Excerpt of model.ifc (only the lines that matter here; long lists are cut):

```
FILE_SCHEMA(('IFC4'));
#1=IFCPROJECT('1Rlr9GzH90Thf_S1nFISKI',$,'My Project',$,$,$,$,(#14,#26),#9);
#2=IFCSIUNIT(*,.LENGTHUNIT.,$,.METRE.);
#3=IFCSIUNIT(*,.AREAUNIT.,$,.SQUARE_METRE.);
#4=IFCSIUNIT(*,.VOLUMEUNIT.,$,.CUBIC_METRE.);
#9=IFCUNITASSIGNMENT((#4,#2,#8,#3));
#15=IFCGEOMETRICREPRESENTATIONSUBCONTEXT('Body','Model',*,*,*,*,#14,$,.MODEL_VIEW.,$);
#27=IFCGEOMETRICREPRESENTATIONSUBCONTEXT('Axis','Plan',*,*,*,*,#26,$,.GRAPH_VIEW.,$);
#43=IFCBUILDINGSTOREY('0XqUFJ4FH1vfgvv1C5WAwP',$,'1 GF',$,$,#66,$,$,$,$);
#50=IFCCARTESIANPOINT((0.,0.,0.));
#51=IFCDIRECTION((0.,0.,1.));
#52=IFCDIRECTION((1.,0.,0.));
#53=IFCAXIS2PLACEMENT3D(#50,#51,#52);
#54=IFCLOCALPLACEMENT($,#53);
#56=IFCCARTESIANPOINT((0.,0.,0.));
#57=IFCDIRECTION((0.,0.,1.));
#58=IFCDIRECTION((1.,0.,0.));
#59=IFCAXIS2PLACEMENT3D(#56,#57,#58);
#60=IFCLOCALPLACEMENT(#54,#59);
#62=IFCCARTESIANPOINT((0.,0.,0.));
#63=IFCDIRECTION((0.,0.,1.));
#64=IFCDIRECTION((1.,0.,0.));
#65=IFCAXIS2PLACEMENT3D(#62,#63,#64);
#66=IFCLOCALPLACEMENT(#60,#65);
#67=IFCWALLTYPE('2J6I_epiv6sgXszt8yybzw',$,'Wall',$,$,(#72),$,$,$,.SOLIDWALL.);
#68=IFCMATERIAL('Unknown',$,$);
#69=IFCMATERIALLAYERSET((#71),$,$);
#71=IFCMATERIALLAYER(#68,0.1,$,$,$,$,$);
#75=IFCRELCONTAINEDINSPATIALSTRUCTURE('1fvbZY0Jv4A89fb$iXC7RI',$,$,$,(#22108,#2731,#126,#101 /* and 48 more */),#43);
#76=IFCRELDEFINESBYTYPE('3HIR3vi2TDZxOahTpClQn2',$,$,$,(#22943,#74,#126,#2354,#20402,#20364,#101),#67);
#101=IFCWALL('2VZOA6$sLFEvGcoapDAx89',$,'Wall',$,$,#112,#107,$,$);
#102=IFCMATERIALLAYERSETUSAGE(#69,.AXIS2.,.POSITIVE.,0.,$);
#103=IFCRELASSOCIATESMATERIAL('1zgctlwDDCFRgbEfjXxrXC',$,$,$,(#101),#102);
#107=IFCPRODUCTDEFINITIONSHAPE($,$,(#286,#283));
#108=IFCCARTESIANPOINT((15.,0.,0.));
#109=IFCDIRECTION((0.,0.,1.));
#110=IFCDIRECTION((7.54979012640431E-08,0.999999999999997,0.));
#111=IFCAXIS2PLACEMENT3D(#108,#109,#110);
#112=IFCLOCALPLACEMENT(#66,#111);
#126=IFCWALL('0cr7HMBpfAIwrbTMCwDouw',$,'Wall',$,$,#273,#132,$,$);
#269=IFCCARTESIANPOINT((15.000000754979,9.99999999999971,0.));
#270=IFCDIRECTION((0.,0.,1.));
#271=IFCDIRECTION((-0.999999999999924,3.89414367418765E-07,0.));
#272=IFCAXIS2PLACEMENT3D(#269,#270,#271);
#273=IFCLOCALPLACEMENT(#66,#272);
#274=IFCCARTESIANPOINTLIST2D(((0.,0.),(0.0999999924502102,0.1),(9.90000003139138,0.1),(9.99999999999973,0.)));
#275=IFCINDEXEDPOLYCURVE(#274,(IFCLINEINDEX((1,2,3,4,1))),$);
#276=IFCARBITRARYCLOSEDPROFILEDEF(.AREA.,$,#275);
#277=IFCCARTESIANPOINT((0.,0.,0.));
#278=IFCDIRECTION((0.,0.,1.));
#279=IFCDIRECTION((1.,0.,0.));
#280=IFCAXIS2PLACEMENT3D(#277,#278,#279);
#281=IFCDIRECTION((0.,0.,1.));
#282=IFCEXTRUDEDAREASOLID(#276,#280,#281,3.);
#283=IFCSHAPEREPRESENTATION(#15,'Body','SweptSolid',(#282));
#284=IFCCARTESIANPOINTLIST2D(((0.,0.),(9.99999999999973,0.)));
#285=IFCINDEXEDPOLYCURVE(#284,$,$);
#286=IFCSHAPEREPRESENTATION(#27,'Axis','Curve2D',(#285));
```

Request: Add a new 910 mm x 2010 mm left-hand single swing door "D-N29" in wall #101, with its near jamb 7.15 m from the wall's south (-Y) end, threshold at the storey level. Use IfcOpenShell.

```python
import numpy as np
import ifcopenshell
import ifcopenshell.api.feature
import ifcopenshell.api.geometry
import ifcopenshell.api.root
import ifcopenshell.api.spatial
import ifcopenshell.geom
import ifcopenshell.util.element
import ifcopenshell.util.placement
import ifcopenshell.util.representation
import ifcopenshell.util.shape
import ifcopenshell.util.unit

model = ifcopenshell.open("model.ifc")
unit_scale = ifcopenshell.util.unit.calculate_unit_scale(model)
settings = ifcopenshell.geom.settings()


def volume(element):
    """Net volume in cubic metres, openings subtracted."""
    shape = ifcopenshell.geom.create_shape(settings, element)
    return ifcopenshell.util.shape.get_volume(shape.geometry)


wall = model.by_guid("2VZOA6$sLFEvGcoapDAx89")
storey = ifcopenshell.util.element.get_container(wall, ifc_class="IfcBuildingStorey")
context = ifcopenshell.util.representation.get_context(model, "Model", "Body", "MODEL_VIEW")
before = volume(wall)

width, height, from_end, sill = 0.91, 2.01, 7.15, 0.0  # metres

# The wall runs along its own X axis, and the end named is its -X end.
wall_shape = ifcopenshell.geom.create_shape(settings, wall)
x, y, z = ifcopenshell.util.shape.get_vertices(wall_shape.geometry).T
start = x.min() + from_end
face, thickness = float(y.min()), float(y.max() - y.min())
wall_matrix = ifcopenshell.util.placement.get_local_placement(wall.ObjectPlacement)
level = ifcopenshell.util.placement.get_local_placement(storey.ObjectPlacement)[2, 3]


def in_wall(x, y):
    """Placement at x, y metres in the wall's axes, at sill height."""
    matrix = wall_matrix.copy()
    matrix[:, 3] = wall_matrix @ np.array([x / unit_scale, y / unit_scale, 0.0, 1.0])
    matrix[2, 3] = level + sill / unit_scale
    return matrix


# Opening: a box that overshoots both wall faces by 50 mm.
opening = ifcopenshell.api.root.create_entity(model, ifc_class="IfcOpeningElement", predefined_type="OPENING")
box = ifcopenshell.api.geometry.add_wall_representation(
    model, context=context, length=width, height=height, thickness=thickness + 0.1
)
ifcopenshell.api.geometry.assign_representation(model, product=opening, representation=box)
ifcopenshell.api.geometry.edit_object_placement(model, product=opening, matrix=in_wall(start, face - 0.05), is_si=False)
ifcopenshell.api.feature.add_feature(model, feature=opening, element=wall)

door = ifcopenshell.api.root.create_entity(model, ifc_class="IfcDoor", name="D-N29", predefined_type="DOOR")
door.OverallWidth, door.OverallHeight = width / unit_scale, height / unit_scale
door.OperationType = "SINGLE_SWING_LEFT"
body = ifcopenshell.api.geometry.add_door_representation(
    model,
    context=context,
    overall_width=door.OverallWidth,
    overall_height=door.OverallHeight,
    operation_type="SINGLE_SWING_LEFT",
    lining_properties={"LiningDepth": thickness / unit_scale, "ThresholdDepth": thickness / unit_scale},
)
ifcopenshell.api.geometry.assign_representation(model, product=door, representation=body)
ifcopenshell.api.spatial.assign_container(model, products=[door], relating_structure=storey)
ifcopenshell.api.feature.add_filling(model, opening=opening, element=door)

# The lining spans the wall, so the door starts at the wall face.
ifcopenshell.api.geometry.edit_object_placement(model, product=door, matrix=in_wall(start, face), is_si=False)

after = volume(wall)

print(f"wall volume {before:.3f} -> {after:.3f} m3")

model.write("model_v2.ifc")
```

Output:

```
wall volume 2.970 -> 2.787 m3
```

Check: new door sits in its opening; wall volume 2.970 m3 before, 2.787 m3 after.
